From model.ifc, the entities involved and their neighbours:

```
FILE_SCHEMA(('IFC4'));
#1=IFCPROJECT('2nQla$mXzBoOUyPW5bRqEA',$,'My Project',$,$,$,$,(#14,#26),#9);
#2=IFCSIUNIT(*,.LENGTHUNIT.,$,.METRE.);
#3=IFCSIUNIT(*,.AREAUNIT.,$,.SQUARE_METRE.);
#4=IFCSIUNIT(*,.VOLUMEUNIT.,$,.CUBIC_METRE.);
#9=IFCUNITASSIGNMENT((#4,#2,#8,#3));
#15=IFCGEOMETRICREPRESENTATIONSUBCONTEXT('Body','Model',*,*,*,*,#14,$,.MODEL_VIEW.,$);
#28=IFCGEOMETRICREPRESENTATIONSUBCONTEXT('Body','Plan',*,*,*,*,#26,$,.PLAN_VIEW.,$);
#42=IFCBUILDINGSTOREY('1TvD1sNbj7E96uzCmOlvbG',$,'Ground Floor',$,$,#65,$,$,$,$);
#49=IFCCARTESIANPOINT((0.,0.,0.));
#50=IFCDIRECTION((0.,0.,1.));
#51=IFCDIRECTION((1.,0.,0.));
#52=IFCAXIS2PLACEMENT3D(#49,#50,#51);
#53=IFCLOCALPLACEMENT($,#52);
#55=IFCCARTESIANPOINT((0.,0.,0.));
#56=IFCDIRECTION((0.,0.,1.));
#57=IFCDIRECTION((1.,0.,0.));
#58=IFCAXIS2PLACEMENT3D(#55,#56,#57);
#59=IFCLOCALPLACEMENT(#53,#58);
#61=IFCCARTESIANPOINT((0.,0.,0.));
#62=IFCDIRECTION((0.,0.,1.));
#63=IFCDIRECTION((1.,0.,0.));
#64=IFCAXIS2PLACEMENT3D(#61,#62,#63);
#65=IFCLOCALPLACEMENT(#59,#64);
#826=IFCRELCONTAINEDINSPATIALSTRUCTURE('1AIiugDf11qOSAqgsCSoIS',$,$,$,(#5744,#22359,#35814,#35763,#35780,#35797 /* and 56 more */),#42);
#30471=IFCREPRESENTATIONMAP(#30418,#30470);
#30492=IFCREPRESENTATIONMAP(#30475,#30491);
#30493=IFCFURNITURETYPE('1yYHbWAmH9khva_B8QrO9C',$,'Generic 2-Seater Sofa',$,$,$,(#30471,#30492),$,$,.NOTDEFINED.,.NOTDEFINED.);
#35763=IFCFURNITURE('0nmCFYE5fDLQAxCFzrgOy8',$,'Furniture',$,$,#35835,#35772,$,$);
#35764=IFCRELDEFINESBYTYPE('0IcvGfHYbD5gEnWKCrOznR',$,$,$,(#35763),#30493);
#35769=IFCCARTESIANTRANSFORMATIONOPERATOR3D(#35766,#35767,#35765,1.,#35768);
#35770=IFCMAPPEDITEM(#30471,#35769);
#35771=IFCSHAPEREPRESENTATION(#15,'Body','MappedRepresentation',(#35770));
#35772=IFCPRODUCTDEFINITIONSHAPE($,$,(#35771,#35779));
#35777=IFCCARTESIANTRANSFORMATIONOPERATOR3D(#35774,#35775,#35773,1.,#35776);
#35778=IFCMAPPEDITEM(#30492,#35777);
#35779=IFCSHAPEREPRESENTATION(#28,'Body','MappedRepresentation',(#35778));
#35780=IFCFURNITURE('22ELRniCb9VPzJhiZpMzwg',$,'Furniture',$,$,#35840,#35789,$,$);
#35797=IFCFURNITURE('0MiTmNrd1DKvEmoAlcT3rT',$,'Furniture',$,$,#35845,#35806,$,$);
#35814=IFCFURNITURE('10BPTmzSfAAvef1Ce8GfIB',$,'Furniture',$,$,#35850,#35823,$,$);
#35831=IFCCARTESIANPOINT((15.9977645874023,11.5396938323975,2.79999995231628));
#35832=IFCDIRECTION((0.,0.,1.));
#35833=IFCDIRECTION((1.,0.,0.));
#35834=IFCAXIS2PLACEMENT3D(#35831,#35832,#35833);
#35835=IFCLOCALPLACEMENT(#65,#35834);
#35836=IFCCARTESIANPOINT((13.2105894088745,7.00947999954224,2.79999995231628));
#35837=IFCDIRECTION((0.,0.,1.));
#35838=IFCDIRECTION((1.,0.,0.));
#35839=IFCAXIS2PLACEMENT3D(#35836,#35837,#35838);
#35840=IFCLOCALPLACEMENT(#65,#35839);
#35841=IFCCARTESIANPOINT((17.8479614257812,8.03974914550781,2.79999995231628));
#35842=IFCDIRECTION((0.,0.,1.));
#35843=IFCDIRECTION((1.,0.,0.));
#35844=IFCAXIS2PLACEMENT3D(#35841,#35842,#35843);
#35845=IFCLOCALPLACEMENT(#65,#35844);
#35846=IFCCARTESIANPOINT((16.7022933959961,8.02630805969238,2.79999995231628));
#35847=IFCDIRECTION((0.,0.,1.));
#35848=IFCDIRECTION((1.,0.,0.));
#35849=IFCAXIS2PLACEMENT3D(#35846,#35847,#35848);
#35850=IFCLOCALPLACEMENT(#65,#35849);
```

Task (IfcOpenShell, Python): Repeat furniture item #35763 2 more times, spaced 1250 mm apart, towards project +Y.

```python
import numpy as np
import ifcopenshell
import ifcopenshell.api.geometry
import ifcopenshell.api.root
import ifcopenshell.util.element
import ifcopenshell.util.placement
import ifcopenshell.util.unit

model = ifcopenshell.open("model.ifc")
unit_scale = ifcopenshell.util.unit.calculate_unit_scale(model)

source = model.by_guid("0nmCFYE5fDLQAxCFzrgOy8")
base = ifcopenshell.util.placement.get_local_placement(source.ObjectPlacement)
step = np.array([0.0, 1.0, 0.0]) * 1.25 / unit_scale

for i in range(1, 3):
    copy = ifcopenshell.api.root.copy_class(model, product=source)
    copy.Representation = ifcopenshell.util.element.copy_deep(
        model, source.Representation, exclude=["IfcGeometricRepresentationContext", "IfcRepresentationMap"]
    )
    matrix = base.copy()
    matrix[:3, 3] += i * step
    print("added at", matrix[:3, 3].round(3) + 0.0)
    ifcopenshell.api.geometry.edit_object_placement(model, product=copy, matrix=matrix, is_si=False)

model.write("model_v2.ifc")
```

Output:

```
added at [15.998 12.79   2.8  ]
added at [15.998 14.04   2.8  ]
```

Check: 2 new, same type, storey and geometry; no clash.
